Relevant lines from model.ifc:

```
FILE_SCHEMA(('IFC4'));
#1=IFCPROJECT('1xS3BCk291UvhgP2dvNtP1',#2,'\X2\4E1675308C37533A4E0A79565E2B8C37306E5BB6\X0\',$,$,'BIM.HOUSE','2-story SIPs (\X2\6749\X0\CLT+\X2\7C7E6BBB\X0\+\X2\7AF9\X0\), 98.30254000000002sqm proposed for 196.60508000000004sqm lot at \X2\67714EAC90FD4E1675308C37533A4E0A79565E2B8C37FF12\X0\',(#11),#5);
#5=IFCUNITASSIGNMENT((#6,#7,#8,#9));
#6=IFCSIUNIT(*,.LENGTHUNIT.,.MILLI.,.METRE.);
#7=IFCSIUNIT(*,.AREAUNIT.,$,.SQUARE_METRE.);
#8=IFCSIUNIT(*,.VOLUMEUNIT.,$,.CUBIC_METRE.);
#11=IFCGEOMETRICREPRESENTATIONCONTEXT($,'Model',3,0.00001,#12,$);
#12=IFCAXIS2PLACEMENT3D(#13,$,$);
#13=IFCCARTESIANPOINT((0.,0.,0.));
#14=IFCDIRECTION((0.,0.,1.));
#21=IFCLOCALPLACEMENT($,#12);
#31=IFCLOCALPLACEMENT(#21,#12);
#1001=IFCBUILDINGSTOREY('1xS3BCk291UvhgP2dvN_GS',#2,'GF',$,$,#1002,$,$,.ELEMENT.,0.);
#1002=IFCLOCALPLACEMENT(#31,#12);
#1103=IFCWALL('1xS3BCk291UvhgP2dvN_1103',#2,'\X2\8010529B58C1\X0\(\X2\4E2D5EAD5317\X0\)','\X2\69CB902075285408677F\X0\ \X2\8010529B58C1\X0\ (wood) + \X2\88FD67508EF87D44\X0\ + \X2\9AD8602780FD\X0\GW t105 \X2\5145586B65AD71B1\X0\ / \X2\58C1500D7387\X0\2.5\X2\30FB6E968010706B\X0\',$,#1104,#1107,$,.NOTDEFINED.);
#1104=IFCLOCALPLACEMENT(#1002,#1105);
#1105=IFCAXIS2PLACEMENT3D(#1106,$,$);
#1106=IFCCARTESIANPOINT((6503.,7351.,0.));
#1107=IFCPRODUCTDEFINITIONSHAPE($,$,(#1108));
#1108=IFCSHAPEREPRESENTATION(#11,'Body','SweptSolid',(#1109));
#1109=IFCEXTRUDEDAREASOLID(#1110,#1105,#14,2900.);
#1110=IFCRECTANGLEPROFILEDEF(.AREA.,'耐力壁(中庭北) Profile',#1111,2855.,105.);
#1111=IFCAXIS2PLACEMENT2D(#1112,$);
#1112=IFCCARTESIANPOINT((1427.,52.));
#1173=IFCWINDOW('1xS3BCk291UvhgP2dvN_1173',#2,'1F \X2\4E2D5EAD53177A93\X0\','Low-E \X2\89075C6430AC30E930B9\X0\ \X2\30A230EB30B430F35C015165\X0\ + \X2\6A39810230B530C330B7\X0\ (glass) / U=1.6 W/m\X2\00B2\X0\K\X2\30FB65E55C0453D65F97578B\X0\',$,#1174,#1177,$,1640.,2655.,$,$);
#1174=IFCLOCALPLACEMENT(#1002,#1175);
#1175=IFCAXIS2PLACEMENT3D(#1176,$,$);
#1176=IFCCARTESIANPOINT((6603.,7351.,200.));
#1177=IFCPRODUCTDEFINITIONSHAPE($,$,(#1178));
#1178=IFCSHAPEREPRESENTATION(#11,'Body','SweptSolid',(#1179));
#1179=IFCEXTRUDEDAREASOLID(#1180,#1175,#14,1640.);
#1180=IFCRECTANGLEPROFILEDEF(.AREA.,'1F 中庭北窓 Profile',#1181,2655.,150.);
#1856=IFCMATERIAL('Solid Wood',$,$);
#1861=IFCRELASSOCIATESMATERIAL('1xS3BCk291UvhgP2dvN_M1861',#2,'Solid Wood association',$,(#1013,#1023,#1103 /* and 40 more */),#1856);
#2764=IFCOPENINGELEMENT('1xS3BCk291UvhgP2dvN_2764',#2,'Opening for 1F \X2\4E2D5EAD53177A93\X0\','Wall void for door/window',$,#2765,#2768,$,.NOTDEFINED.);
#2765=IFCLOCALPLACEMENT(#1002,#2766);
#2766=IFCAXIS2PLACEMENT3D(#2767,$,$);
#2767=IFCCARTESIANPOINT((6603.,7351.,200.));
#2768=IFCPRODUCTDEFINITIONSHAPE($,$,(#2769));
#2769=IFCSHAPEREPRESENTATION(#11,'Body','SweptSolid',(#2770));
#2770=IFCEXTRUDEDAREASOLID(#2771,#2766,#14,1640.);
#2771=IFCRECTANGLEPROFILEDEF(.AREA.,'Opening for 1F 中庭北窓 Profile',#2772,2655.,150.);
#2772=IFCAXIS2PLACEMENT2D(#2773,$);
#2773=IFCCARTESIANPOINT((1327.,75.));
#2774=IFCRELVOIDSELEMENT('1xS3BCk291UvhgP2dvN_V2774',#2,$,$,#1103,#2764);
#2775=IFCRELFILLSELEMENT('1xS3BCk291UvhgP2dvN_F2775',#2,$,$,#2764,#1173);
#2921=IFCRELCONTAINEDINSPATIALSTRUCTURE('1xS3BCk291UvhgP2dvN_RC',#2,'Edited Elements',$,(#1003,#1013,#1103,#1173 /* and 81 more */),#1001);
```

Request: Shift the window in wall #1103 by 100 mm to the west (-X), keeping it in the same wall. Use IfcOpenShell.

```python
import ifcopenshell
import ifcopenshell.api.geometry
import ifcopenshell.util.placement

model = ifcopenshell.open("model.ifc")

window = model.by_guid("1xS3BCk291UvhgP2dvN_1173")
opening = window.FillsVoids[0].RelatingOpeningElement
wall = opening.VoidsElements[0].RelatingBuildingElement

wall_matrix = ifcopenshell.util.placement.get_local_placement(wall.ObjectPlacement)
shift = wall_matrix[:3, 0] * -100.0
before = ifcopenshell.util.placement.get_local_placement(window.ObjectPlacement)[:3, 3].copy()

# The window is not placed relative to its opening, so move both.
for product in (opening, window):
    matrix = ifcopenshell.util.placement.get_local_placement(product.ObjectPlacement)
    matrix[:3, 3] += shift
    ifcopenshell.api.geometry.edit_object_placement(model, product=product, matrix=matrix, is_si=False)

after = ifcopenshell.util.placement.get_local_placement(window.ObjectPlacement)[:3, 3]
print("window moved by", (after - before).round(3) + 0.0)

model.write("model-out.ifc")
```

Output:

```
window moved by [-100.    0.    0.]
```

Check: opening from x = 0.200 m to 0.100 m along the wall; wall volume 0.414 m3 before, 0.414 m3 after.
